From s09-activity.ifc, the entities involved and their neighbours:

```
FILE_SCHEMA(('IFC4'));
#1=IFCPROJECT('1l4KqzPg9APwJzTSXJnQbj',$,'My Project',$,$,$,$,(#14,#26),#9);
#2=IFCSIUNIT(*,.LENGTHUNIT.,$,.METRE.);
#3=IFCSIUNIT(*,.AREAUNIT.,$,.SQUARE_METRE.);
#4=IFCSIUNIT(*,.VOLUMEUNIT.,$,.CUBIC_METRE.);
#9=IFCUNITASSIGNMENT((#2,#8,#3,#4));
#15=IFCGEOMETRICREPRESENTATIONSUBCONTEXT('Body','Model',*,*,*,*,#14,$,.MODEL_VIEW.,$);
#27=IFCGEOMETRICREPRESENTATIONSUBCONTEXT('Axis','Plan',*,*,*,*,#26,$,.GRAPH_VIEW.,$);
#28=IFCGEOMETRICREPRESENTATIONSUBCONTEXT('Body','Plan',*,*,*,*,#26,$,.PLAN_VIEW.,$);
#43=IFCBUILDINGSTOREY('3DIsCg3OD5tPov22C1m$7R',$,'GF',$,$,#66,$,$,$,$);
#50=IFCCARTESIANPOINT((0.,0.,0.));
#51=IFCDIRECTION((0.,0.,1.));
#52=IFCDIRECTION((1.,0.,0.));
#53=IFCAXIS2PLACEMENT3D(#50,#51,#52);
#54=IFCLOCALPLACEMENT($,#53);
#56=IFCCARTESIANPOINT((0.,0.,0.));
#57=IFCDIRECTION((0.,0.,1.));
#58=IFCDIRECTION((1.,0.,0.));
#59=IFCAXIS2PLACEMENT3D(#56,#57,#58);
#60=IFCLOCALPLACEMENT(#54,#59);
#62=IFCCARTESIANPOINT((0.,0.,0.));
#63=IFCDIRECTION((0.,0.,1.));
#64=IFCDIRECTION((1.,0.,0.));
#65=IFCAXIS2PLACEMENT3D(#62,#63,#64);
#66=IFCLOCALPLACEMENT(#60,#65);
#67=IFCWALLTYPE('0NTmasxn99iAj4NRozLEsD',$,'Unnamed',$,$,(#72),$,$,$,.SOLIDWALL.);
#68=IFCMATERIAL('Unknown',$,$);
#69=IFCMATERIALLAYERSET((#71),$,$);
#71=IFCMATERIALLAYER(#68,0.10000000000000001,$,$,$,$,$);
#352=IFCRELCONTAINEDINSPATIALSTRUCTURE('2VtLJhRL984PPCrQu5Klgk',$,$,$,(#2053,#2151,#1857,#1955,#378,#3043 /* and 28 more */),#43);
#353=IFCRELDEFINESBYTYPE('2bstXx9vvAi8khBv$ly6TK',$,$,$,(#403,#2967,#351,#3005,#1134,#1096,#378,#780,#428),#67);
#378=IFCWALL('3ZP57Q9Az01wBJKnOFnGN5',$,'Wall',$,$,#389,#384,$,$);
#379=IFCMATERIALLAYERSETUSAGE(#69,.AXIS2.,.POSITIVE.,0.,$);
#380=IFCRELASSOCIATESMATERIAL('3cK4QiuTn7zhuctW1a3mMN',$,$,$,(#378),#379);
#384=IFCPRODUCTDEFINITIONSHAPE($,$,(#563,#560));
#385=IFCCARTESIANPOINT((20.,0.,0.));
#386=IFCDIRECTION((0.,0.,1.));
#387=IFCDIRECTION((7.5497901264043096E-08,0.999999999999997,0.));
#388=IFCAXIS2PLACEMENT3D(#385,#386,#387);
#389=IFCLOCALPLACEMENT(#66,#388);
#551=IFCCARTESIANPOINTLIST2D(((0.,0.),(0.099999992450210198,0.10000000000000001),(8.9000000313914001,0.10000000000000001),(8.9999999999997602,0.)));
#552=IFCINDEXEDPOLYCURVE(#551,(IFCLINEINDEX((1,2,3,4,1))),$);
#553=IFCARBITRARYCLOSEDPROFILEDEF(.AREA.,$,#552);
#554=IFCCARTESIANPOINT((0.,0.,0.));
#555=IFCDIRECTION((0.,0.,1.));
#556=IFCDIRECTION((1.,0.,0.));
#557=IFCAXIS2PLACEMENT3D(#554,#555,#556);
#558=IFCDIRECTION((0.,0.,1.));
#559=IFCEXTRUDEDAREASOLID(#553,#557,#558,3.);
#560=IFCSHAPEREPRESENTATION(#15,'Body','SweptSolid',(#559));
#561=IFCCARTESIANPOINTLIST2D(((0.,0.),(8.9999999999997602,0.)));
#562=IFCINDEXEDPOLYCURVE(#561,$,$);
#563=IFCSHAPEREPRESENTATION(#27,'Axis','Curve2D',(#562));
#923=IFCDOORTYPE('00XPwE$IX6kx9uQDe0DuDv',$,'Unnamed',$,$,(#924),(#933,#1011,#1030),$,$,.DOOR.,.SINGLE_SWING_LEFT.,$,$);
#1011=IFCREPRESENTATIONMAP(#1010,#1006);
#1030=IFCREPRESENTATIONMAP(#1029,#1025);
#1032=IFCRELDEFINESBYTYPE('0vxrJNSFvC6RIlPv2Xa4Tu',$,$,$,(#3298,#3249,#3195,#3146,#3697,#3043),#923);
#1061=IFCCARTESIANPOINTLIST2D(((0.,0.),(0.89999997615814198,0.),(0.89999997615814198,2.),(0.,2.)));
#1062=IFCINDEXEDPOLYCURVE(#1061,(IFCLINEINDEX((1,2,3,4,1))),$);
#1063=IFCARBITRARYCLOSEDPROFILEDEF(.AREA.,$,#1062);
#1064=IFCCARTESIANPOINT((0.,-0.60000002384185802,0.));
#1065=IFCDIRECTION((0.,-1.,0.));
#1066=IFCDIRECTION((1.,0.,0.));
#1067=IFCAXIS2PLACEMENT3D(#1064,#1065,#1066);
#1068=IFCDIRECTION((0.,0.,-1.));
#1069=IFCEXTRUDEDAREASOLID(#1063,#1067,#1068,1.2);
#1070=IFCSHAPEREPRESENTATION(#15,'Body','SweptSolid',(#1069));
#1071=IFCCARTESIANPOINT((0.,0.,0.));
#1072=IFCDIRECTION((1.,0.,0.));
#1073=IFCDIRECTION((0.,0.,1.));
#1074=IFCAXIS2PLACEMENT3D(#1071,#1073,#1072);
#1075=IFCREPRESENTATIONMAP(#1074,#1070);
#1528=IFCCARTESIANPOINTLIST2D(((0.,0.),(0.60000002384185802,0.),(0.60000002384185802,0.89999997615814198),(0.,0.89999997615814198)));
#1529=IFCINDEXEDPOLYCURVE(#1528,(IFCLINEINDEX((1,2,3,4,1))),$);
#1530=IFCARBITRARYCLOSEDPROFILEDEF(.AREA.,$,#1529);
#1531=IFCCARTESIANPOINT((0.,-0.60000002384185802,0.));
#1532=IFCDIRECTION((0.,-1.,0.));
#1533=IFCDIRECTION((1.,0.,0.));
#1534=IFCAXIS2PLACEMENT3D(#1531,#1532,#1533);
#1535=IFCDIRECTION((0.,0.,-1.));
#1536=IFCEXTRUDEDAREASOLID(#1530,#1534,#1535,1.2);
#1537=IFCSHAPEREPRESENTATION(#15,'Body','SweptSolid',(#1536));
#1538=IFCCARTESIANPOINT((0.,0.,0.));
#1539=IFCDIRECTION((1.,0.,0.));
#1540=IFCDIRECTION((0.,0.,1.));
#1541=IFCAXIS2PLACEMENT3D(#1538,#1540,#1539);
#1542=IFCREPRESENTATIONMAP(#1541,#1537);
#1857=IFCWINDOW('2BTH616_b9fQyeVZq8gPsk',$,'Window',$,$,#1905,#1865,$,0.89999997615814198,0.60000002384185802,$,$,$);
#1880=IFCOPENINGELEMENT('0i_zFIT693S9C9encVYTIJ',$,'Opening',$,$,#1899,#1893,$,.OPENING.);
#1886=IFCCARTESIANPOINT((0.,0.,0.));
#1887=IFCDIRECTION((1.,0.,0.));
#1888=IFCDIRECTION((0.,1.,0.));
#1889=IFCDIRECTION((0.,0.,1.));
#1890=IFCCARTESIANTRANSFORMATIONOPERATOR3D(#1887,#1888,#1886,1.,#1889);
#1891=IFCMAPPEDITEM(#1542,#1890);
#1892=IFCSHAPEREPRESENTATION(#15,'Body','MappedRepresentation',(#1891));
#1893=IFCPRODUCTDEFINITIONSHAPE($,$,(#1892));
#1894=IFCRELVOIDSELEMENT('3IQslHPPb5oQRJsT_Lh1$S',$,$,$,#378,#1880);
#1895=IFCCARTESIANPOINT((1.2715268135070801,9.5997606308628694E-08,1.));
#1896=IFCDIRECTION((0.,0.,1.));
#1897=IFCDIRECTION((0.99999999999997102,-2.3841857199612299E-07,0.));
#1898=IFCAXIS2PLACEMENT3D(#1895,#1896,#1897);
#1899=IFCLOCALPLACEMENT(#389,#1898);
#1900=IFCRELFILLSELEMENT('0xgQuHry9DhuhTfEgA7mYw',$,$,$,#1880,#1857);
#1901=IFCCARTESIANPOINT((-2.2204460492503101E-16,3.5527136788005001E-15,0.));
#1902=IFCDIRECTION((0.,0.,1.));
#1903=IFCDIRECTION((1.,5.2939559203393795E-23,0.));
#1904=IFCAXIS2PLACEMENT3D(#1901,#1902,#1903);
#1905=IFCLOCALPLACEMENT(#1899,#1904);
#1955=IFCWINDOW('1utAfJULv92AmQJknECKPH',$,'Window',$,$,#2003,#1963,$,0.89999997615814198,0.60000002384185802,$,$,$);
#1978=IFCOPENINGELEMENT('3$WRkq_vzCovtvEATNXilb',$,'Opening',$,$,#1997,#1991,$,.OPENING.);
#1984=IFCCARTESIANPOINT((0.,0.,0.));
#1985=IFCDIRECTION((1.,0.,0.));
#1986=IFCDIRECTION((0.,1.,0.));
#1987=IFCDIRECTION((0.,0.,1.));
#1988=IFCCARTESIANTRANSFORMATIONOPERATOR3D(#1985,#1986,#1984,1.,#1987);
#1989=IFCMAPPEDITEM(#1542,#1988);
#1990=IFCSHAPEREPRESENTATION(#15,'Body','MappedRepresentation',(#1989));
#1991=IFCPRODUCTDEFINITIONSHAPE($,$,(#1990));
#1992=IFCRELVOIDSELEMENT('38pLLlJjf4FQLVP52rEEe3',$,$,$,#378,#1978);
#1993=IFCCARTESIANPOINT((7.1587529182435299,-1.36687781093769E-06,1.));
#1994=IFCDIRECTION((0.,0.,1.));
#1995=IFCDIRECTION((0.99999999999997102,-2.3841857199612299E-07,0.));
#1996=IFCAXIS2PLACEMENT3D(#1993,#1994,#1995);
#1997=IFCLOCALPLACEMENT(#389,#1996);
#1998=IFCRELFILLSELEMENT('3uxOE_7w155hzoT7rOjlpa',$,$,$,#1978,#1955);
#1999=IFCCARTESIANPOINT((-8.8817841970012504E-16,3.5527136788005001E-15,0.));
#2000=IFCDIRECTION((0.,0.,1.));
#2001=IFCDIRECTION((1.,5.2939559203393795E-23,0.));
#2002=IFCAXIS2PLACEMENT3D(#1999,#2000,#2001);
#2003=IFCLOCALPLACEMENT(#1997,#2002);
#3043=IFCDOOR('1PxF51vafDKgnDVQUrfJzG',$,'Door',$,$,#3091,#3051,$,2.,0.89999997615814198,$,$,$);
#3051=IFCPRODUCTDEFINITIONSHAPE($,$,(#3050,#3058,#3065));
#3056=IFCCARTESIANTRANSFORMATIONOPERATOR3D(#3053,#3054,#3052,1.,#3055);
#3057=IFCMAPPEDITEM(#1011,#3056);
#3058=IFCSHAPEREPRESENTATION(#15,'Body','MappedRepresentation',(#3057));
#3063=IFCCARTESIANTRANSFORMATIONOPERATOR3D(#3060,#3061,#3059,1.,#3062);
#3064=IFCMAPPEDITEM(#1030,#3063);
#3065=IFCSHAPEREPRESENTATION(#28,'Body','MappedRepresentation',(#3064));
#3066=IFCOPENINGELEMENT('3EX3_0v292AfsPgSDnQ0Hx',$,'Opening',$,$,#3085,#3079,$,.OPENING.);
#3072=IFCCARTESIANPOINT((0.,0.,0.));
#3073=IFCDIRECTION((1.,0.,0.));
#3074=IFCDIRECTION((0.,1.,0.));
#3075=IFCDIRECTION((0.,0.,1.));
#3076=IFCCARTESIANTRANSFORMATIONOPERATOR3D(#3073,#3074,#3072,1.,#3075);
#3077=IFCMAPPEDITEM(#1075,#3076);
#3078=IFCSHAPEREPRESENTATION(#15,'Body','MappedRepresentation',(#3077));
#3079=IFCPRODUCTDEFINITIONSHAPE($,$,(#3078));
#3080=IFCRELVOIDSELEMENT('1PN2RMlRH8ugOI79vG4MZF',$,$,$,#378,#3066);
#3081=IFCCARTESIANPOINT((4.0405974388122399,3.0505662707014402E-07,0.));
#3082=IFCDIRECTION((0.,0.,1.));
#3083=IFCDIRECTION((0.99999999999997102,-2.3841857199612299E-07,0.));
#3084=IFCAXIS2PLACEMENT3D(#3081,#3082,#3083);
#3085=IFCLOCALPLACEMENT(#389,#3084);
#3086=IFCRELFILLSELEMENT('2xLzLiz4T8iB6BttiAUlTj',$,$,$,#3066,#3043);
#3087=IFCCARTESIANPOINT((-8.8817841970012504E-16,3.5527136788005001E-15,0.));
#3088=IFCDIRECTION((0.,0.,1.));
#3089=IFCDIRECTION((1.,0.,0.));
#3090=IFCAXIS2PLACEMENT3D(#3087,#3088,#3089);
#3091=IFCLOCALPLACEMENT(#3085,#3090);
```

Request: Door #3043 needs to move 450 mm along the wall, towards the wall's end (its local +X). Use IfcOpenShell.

```python
import ifcopenshell
import ifcopenshell.api.geometry
import ifcopenshell.util.placement
import ifcopenshell.util.unit

model = ifcopenshell.open("s09-activity.ifc")
unit_scale = ifcopenshell.util.unit.calculate_unit_scale(model)

door = model.by_guid("1PxF51vafDKgnDVQUrfJzG")
opening = door.FillsVoids[0].RelatingOpeningElement
wall = opening.VoidsElements[0].RelatingBuildingElement

wall_matrix = ifcopenshell.util.placement.get_local_placement(wall.ObjectPlacement)
shift = wall_matrix[:3, 0] * 0.45 / unit_scale
before = ifcopenshell.util.placement.get_local_placement(door.ObjectPlacement)[:3, 3].copy()

# The door is placed relative to its opening, so it follows when the opening moves.
matrix = ifcopenshell.util.placement.get_local_placement(opening.ObjectPlacement)
matrix[:3, 3] += shift
ifcopenshell.api.geometry.edit_object_placement(
    model, product=opening, matrix=matrix, is_si=False, should_transform_children=True
)

after = ifcopenshell.util.placement.get_local_placement(door.ObjectPlacement)[:3, 3]
print("door moved by", (after - before).round(3) + 0.0)

model.write("s09-activity-out.ifc")
```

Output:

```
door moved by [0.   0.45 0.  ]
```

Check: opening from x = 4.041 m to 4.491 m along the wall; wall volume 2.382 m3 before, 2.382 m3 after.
